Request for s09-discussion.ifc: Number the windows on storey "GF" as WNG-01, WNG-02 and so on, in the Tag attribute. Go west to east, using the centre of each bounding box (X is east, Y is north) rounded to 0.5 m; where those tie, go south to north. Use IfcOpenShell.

First a look at what the model holds.

```python
import ifcopenshell
import ifcopenshell.util.element
import ifcopenshell.util.placement

model = ifcopenshell.open("s09-discussion.ifc")
print(model.schema)
storey = next(s for s in model.by_type("IfcBuildingStorey") if s.Name == "GF")
windows = [e for e in ifcopenshell.util.element.get_decomposition(storey) if e.is_a("IfcWindow")]
for e in sorted(windows, key=lambda e: e.id()):
    origin = ifcopenshell.util.placement.get_local_placement(e.ObjectPlacement)[:3, 3]
    print(e.id(), e.Tag, e.Name, origin.round(2) + 0.0, sep=" | ")
```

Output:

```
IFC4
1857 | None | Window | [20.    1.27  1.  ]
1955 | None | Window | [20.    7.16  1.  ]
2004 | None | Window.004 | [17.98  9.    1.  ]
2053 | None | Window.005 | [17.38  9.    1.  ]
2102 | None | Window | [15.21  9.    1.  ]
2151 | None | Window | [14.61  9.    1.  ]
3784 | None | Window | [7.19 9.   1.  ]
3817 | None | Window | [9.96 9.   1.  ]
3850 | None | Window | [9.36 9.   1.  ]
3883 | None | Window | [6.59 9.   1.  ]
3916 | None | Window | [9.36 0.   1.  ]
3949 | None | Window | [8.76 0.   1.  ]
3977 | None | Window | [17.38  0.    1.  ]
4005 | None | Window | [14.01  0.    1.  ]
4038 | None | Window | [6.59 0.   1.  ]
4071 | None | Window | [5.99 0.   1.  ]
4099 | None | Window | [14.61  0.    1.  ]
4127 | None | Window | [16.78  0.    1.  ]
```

```python
import ifcopenshell
import ifcopenshell.geom
import ifcopenshell.util.element
import ifcopenshell.util.shape

model = ifcopenshell.open("s09-discussion.ifc")
settings = ifcopenshell.geom.settings()
settings.set("use-world-coords", True)


def centre(element):
    shape = ifcopenshell.geom.create_shape(settings, element)
    return ifcopenshell.util.shape.get_bbox_centroid(shape.geometry)


storey = next(s for s in model.by_type("IfcBuildingStorey") if s.Name == "GF")
windows = [e for e in ifcopenshell.util.element.get_decomposition(storey) if e.is_a("IfcWindow")]

# Insertion points can sit at a corner or the storey origin, so sort by the geometry (in metres).
centres = {e: centre(e) for e in windows}
windows.sort(key=lambda e: (round(centres[e][0] / 0.5), centres[e][1]))

for i, e in enumerate(windows, start=1):
    number = f"WNG-{i:02d}"
    e.Tag = number
    print(e.id(), number)

model.write("s09-discussion_v2.ifc")
```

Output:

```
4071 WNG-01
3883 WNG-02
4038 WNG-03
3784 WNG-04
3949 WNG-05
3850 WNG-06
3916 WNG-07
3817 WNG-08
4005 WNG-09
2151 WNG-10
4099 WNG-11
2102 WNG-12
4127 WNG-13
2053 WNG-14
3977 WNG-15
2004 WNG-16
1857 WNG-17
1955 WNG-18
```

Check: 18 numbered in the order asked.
